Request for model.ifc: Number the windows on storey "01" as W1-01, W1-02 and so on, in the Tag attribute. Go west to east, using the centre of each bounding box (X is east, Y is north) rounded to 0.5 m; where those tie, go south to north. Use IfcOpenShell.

First a look at what the model holds.

```python
import ifcopenshell
import ifcopenshell.util.element
import ifcopenshell.util.placement

model = ifcopenshell.open("model.ifc")
print(model.schema)
storey = next(s for s in model.by_type("IfcBuildingStorey") if s.Name == "01")
windows = [e for e in ifcopenshell.util.element.get_decomposition(storey) if e.is_a("IfcWindow")]
for e in sorted(windows, key=lambda e: e.id()):
    origin = ifcopenshell.util.placement.get_local_placement(e.ObjectPlacement)[:3, 3]
    print(e.id(), e.Tag, e.Name, origin.round(2) + 0.0, sep=" | ")
```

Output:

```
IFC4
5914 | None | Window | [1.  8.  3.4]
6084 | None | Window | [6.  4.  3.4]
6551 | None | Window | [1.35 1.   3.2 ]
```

```python
import ifcopenshell
import ifcopenshell.geom
import ifcopenshell.util.element
import ifcopenshell.util.shape

model = ifcopenshell.open("model.ifc")
settings = ifcopenshell.geom.settings()
settings.set("use-world-coords", True)


def centre(element):
    shape = ifcopenshell.geom.create_shape(settings, element)
    return ifcopenshell.util.shape.get_bbox_centroid(shape.geometry)


storey = next(s for s in model.by_type("IfcBuildingStorey") if s.Name == "01")
windows = [e for e in ifcopenshell.util.element.get_decomposition(storey) if e.is_a("IfcWindow")]

# Insertion points can sit at a corner or the storey origin, so sort by the geometry (in metres).
centres = {e: centre(e) for e in windows}
windows.sort(key=lambda e: (round(centres[e][0] / 0.5), centres[e][1]))

for i, e in enumerate(windows, start=1):
    number = f"W1-{i:02d}"
    e.Tag = number
    print(e.id(), number)

model.write("model_rev.ifc")
```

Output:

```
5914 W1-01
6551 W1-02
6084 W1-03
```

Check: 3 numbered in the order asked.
